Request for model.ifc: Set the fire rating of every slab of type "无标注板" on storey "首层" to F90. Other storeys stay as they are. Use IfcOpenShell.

First a look at what the model holds.

```python
import ifcopenshell
import ifcopenshell.util.element

model = ifcopenshell.open("model.ifc")
print(model.schema)
storey = next(s for s in model.by_type("IfcBuildingStorey") if s.Name == "首层")
slabs = [e for e in ifcopenshell.util.element.get_decomposition(storey) if e.is_a("IfcSlab")]
seen = {}
for e in slabs:
    element_type = ifcopenshell.util.element.get_type(e)
    key = (element_type.Name if element_type != e and element_type else None, ifcopenshell.util.element.get_pset(e, "Pset_SlabCommon", "FireRating"))
    seen[key] = seen.get(key, 0) + 1
for (name, value), count in sorted(seen.items(), key=str):
    print(count, "x", name, "|", value)
```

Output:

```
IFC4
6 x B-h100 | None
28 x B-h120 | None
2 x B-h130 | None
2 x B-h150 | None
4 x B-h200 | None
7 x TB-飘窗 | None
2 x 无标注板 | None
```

```python
import ifcopenshell
import ifcopenshell.api.pset
import ifcopenshell.util.element

model = ifcopenshell.open("model.ifc")

storey = next(s for s in model.by_type("IfcBuildingStorey") if s.Name == "首层")
slabs = [e for e in ifcopenshell.util.element.get_decomposition(storey) if e.is_a("IfcSlab")]

count = 0
for e in slabs:
    element_type = ifcopenshell.util.element.get_type(e)
    if element_type in (None, e) or element_type.Name != "无标注板":
        continue
    # add_pset returns the element's existing set when there is one.
    pset = ifcopenshell.api.pset.add_pset(model, product=e, name="Pset_SlabCommon")
    ifcopenshell.api.pset.edit_pset(model, pset=pset, properties={"FireRating": "F90"})
    count += 1

print(count, "slabs updated")

model.write("model_v2.ifc")
```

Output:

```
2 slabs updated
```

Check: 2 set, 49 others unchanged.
